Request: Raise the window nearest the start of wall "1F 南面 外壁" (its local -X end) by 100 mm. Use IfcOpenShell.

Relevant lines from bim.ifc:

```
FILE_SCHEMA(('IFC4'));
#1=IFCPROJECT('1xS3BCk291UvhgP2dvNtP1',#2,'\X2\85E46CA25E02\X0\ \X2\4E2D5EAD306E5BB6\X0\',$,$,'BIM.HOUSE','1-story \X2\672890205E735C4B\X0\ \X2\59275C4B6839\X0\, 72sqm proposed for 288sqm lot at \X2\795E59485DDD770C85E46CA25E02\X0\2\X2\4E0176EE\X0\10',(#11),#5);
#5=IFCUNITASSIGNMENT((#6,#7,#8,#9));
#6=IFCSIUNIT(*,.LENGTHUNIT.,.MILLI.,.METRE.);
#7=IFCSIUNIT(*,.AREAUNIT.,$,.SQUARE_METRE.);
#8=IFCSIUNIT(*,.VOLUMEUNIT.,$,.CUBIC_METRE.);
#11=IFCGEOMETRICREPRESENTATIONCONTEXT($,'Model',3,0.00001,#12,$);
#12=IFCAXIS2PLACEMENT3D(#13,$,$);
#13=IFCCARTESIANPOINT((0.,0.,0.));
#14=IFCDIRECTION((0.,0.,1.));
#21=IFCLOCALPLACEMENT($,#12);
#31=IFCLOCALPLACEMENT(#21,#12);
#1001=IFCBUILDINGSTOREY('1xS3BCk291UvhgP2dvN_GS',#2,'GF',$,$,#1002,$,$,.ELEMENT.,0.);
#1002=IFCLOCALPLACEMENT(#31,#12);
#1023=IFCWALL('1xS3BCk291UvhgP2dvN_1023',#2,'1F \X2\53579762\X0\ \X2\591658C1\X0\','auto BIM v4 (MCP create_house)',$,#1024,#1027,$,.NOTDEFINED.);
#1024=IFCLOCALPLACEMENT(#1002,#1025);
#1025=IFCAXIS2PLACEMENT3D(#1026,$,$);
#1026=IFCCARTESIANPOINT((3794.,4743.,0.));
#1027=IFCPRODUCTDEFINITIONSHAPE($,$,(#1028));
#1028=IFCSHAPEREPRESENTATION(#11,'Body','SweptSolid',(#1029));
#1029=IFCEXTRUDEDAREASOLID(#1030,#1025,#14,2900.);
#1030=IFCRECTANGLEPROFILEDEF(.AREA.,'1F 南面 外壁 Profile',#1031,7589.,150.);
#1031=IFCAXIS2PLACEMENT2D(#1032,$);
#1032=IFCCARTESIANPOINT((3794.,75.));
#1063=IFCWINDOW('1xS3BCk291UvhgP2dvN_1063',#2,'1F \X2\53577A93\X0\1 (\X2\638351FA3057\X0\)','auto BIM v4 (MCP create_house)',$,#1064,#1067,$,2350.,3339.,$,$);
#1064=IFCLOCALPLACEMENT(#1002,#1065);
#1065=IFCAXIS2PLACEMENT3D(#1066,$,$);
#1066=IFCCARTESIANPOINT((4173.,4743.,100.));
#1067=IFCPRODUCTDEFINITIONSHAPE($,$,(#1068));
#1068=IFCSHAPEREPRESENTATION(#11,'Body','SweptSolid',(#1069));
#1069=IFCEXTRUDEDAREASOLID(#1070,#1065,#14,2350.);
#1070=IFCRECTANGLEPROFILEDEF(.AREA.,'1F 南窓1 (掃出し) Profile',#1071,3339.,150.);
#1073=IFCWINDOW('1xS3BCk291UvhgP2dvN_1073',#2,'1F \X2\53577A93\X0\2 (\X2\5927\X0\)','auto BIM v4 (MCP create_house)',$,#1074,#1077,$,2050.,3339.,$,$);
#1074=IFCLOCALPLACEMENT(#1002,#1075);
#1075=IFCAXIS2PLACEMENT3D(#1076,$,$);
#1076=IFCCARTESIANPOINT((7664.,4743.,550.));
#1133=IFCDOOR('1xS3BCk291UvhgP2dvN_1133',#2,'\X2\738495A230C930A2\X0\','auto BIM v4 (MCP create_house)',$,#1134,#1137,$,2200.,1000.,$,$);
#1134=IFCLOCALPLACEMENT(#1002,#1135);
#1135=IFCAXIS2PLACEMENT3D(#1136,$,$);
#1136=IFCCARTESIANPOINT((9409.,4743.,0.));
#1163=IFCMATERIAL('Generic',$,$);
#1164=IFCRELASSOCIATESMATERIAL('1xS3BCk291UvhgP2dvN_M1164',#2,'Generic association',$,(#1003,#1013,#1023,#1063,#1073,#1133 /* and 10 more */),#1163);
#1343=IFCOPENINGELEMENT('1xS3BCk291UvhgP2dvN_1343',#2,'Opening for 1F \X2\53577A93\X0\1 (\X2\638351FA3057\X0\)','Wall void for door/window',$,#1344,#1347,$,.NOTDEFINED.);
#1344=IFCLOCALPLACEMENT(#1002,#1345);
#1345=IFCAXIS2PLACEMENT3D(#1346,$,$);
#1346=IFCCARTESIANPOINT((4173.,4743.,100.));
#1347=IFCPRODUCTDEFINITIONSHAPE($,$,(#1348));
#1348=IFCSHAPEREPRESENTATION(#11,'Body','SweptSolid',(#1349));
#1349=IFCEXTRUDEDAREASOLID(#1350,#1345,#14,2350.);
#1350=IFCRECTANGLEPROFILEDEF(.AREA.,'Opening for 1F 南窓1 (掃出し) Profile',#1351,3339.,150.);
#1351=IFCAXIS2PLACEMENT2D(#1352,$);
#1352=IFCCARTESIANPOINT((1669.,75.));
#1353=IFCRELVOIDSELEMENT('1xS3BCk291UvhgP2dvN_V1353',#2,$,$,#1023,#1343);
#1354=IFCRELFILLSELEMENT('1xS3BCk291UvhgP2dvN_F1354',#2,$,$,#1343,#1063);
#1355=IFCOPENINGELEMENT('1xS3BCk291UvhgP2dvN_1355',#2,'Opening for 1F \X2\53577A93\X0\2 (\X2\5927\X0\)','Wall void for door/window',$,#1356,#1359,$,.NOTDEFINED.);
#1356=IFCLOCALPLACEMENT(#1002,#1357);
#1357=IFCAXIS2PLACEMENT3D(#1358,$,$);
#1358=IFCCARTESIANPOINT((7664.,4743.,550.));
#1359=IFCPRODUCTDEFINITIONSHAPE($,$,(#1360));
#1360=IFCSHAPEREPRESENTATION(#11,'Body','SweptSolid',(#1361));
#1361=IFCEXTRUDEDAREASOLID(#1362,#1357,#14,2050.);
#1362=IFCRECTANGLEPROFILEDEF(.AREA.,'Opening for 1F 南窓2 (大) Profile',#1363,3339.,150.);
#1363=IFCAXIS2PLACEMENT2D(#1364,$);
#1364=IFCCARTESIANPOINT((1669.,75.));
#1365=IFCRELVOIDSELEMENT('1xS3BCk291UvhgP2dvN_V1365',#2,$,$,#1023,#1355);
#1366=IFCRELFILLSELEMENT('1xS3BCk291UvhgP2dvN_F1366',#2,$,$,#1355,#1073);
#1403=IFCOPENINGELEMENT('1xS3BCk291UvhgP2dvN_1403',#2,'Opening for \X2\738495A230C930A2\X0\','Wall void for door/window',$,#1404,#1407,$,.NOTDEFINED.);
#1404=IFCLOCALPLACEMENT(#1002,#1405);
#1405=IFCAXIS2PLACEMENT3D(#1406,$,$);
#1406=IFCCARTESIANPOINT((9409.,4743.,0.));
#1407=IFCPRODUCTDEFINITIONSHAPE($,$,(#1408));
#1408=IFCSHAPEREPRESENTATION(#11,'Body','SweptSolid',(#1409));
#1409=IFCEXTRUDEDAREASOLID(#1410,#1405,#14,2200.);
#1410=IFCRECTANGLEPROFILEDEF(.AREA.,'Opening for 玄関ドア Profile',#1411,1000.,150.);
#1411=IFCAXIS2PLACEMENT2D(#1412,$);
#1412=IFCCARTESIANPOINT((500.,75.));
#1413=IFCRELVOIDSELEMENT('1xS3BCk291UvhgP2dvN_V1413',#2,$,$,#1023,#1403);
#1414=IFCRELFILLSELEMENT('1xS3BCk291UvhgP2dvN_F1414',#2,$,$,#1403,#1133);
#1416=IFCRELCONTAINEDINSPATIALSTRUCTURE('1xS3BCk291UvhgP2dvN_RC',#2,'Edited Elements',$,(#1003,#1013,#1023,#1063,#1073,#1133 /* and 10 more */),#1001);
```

```python
import numpy as np
import ifcopenshell
import ifcopenshell.api.geometry
import ifcopenshell.util.placement
import ifcopenshell.util.unit

model = ifcopenshell.open("bim.ifc")
unit_scale = ifcopenshell.util.unit.calculate_unit_scale(model)

window = model.by_guid("1xS3BCk291UvhgP2dvN_1063")
opening = window.FillsVoids[0].RelatingOpeningElement
dz = 100.0

shift = np.array([0.0, 0.0, dz])
# The window is not placed relative to its opening, so move both.
for product in (opening, window):
    matrix = ifcopenshell.util.placement.get_local_placement(product.ObjectPlacement)
    matrix[:3, 3] += shift
    ifcopenshell.api.geometry.edit_object_placement(model, product=product, matrix=matrix, is_si=False)

print(f"moved by {dz * unit_scale:+.3f} m")

model.write("bim_updated.ifc")
```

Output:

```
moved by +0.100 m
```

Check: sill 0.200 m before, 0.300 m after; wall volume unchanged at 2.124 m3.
